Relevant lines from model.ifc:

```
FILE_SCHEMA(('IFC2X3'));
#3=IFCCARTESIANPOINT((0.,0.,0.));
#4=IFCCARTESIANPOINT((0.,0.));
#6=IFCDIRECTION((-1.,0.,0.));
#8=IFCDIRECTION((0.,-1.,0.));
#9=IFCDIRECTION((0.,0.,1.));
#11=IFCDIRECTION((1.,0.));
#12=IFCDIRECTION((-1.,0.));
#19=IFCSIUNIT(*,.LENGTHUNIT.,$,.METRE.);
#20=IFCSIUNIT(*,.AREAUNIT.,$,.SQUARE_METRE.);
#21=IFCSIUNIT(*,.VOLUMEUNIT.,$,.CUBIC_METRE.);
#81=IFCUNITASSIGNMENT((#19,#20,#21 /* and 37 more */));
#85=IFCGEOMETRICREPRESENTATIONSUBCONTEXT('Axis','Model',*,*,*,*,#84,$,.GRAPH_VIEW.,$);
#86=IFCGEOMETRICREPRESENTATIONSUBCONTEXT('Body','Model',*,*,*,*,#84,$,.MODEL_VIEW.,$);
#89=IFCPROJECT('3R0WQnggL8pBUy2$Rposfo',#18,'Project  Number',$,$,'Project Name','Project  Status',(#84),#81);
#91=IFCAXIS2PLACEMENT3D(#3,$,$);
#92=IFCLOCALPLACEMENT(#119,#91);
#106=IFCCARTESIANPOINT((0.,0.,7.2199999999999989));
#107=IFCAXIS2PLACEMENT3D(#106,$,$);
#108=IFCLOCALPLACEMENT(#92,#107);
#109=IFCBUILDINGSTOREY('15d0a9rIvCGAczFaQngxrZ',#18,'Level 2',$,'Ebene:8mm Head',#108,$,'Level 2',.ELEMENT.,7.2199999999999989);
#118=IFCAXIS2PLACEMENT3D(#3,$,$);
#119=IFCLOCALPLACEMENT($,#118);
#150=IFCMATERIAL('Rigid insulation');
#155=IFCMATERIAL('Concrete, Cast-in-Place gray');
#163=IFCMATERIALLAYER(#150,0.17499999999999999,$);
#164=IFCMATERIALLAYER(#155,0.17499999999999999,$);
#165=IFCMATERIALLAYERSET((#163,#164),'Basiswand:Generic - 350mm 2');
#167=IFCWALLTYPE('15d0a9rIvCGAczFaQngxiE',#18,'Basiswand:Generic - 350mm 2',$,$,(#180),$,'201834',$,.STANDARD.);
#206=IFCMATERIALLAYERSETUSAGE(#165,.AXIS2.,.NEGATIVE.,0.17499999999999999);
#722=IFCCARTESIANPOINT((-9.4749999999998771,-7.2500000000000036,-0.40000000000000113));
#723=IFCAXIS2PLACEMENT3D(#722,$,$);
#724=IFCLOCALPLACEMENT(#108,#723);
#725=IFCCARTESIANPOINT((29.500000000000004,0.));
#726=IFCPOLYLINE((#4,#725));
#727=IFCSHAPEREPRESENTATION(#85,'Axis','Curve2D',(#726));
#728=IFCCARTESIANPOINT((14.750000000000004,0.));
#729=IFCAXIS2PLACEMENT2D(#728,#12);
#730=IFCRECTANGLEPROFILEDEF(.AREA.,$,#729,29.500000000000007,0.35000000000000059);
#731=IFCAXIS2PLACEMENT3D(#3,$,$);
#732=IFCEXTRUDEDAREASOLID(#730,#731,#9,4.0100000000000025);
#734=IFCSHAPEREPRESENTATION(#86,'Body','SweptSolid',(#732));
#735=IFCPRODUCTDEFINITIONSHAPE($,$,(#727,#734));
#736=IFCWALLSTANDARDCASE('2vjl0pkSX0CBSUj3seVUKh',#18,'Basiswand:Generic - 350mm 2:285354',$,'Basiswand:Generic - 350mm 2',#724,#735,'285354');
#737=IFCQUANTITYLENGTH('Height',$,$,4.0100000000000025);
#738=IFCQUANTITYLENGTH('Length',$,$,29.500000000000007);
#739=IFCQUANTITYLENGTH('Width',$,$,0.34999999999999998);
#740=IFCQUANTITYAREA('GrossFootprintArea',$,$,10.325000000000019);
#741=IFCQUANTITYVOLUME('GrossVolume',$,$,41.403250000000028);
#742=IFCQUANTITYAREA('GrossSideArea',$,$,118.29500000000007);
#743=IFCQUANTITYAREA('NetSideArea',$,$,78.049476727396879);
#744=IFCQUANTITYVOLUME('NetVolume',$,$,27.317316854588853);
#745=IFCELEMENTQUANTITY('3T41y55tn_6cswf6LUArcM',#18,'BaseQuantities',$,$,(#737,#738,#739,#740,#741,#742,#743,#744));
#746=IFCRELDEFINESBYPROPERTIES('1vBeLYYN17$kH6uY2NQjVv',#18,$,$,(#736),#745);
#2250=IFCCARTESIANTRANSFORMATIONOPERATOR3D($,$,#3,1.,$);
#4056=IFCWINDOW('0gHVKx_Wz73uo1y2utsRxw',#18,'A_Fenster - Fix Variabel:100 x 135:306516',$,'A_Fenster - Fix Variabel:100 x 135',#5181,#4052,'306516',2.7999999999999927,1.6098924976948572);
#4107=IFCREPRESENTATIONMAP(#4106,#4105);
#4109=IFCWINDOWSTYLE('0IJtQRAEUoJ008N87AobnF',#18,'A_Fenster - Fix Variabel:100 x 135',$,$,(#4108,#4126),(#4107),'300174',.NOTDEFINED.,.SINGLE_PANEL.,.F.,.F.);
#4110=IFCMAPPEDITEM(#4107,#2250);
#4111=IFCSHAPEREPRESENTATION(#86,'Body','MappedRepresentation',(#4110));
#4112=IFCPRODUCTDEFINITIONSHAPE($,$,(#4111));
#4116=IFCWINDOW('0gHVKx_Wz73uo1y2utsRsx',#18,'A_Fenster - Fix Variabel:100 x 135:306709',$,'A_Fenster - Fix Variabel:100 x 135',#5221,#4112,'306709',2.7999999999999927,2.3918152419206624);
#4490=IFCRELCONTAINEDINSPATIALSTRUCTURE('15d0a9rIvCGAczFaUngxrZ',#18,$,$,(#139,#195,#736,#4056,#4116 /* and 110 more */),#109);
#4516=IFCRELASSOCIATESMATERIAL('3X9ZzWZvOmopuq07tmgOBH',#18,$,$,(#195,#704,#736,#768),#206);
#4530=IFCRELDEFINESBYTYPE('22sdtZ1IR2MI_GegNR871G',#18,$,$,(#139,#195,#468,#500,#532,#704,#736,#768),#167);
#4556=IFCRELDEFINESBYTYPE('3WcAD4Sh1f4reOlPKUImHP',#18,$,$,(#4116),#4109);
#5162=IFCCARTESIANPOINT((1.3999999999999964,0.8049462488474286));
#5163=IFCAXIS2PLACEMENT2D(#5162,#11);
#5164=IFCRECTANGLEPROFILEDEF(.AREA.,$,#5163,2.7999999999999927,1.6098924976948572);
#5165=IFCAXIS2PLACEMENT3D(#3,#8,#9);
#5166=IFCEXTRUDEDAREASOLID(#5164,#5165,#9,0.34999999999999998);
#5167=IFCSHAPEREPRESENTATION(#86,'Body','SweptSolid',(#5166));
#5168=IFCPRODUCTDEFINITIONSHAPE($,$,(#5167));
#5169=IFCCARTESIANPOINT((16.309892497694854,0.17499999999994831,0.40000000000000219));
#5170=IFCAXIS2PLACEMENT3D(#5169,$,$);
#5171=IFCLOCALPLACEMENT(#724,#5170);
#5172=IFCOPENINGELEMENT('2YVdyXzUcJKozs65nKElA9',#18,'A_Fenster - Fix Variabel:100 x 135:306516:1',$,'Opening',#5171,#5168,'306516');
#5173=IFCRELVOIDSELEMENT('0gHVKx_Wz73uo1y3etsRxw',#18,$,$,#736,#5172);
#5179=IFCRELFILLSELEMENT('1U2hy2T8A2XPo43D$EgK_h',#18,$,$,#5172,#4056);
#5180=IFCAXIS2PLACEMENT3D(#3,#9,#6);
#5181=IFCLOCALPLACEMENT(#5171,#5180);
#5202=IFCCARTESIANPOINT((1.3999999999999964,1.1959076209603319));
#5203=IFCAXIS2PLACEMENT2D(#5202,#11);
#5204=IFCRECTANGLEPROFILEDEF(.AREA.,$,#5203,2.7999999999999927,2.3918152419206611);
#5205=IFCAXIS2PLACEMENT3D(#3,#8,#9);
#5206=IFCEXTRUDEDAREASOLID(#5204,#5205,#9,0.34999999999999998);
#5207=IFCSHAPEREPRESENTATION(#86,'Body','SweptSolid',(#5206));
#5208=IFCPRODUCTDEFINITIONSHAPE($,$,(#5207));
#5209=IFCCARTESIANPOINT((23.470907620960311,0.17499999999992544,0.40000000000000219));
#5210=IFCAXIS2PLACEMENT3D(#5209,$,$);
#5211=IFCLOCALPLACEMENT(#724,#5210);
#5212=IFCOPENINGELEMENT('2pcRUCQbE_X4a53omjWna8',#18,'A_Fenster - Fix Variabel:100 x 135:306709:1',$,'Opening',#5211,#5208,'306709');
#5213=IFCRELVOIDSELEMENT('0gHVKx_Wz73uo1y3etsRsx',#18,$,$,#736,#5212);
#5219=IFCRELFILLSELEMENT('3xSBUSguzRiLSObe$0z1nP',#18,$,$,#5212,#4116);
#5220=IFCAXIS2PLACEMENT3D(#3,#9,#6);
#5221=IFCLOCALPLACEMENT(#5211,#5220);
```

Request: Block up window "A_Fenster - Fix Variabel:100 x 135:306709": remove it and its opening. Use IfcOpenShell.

```python
import ifcopenshell
import ifcopenshell.api.feature
import ifcopenshell.api.pset
import ifcopenshell.api.root
import ifcopenshell.geom
import ifcopenshell.util.element
import ifcopenshell.util.shape
import ifcopenshell.util.unit

model = ifcopenshell.open("model.ifc")
area_scale = ifcopenshell.util.unit.calculate_unit_scale(model, "AREAUNIT")
volume_scale = ifcopenshell.util.unit.calculate_unit_scale(model, "VOLUMEUNIT")
settings = ifcopenshell.geom.settings()


def volume(element):
    """Net volume in cubic metres, openings subtracted."""
    shape = ifcopenshell.geom.create_shape(settings, element)
    return ifcopenshell.util.shape.get_volume(shape.geometry)


window = model.by_guid("0gHVKx_Wz73uo1y2utsRsx")
opening = window.FillsVoids[0].RelatingOpeningElement
wall = opening.VoidsElements[0].RelatingBuildingElement
before = volume(wall)

ifcopenshell.api.root.remove_product(model, product=window)
ifcopenshell.api.feature.remove_feature(model, feature=opening)

after = volume(wall)
thickness = 0.35  # wall thickness in metres

# Update the wall's stored quantities.
qto = model.by_id(ifcopenshell.util.element.get_pset(wall, "BaseQuantities", should_inherit=False)["id"])
ifcopenshell.api.pset.edit_qto(model, qto=qto, properties={
    "NetSideArea": after / thickness / area_scale,
    "NetVolume": after / volume_scale,
})

print(f"wall volume {before:.3f} -> {after:.3f} m3")

model.write("model-out.ifc")
```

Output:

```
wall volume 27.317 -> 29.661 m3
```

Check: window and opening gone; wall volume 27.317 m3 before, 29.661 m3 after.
